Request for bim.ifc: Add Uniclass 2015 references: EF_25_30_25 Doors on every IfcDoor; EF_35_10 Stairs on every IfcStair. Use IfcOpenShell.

First a look at what the model holds.

```python
import ifcopenshell

model = ifcopenshell.open("bim.ifc")
print(model.schema)
print("classifications:", [c.Name for c in model.by_type("IfcClassification")])
for ifc_class in ("IfcDoor", "IfcRoof", "IfcStair", "IfcWall", "IfcWindow"):
    print(ifc_class, len(model.by_type(ifc_class)))
```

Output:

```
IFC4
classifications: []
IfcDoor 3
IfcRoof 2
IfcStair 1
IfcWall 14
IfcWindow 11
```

```python
import ifcopenshell
import ifcopenshell.api.classification

model = ifcopenshell.open("bim.ifc")

system = ifcopenshell.api.classification.add_classification(model, classification="Uniclass 2015")

codes = {
    "IfcDoor": ("EF_25_30_25", "Doors"),
    "IfcStair": ("EF_35_10", "Stairs"),
}
for ifc_class, (code, name) in codes.items():
    products = model.by_type(ifc_class)
    ifcopenshell.api.classification.add_reference(
        model, products=products, classification=system, identification=code, name=name
    )
    print(code, len(products))

model.write("bim_rev.ifc")
```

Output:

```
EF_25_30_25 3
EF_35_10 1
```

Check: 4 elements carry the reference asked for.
